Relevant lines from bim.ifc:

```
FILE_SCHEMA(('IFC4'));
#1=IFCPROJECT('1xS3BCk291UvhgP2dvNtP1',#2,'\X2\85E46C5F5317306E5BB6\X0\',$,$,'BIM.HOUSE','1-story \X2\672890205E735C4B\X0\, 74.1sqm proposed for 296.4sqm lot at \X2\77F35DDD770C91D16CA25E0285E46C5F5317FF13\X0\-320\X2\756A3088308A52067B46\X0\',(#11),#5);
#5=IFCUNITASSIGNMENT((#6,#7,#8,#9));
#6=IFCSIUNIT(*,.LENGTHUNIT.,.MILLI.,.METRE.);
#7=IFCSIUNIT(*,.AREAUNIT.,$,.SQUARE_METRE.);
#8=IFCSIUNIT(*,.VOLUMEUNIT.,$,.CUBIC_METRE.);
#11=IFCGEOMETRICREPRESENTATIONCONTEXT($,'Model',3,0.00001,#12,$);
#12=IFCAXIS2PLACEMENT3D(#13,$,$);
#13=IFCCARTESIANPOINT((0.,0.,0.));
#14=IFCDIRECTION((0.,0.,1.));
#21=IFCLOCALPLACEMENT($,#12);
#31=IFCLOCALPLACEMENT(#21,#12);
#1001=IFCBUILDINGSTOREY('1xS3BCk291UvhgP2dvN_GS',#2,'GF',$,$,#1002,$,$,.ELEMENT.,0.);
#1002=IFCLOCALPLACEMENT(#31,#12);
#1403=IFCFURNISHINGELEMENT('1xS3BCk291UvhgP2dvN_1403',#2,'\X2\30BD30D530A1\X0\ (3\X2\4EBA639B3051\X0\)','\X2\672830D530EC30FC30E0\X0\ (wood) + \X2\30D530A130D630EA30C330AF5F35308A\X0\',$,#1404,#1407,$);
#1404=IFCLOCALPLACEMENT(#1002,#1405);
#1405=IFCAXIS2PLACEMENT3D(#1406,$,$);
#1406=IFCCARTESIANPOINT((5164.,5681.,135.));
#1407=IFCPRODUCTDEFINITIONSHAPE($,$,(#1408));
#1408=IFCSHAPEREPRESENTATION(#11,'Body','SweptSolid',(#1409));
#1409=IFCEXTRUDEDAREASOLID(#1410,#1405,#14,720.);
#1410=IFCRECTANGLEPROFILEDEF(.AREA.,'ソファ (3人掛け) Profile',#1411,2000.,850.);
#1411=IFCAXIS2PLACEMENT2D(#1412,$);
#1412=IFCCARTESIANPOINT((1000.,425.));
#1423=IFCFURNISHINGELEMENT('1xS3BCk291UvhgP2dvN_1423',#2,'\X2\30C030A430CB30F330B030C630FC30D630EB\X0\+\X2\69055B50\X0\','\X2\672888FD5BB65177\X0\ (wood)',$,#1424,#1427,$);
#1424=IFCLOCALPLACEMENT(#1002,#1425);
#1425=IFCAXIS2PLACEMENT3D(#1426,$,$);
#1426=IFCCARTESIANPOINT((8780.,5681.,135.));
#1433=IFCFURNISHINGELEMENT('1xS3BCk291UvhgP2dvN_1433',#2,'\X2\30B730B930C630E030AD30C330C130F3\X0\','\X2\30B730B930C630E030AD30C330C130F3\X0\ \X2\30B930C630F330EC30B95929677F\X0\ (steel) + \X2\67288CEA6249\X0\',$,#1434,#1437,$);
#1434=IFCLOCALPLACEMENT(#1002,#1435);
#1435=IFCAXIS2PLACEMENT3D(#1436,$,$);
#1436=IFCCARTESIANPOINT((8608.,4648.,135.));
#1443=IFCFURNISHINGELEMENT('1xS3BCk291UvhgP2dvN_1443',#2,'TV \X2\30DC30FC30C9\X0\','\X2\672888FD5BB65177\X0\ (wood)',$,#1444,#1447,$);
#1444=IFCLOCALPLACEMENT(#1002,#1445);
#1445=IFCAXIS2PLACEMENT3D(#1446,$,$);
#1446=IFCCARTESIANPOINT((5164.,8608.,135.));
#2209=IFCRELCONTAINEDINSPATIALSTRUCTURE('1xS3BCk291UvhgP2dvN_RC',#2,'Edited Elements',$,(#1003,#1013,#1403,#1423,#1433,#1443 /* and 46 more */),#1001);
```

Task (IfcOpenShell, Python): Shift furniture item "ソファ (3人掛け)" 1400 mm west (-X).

```python
import ifcopenshell
import ifcopenshell.api.geometry
import ifcopenshell.util.placement
import ifcopenshell.util.unit

model = ifcopenshell.open("bim.ifc")
unit_scale = ifcopenshell.util.unit.calculate_unit_scale(model)

item = model.by_id(1403)
matrix = ifcopenshell.util.placement.get_local_placement(item.ObjectPlacement)
matrix[0, 3] -= 1.4 / unit_scale
ifcopenshell.api.geometry.edit_object_placement(model, product=item, matrix=matrix, is_si=False)

print(ifcopenshell.util.placement.get_local_placement(item.ObjectPlacement).round(3) + 0.0)

model.write("bim-out.ifc")
```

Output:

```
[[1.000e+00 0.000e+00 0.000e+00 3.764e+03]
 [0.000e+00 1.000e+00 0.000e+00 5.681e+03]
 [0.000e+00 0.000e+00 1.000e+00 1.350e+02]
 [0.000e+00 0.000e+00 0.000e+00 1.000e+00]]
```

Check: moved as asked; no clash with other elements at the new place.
